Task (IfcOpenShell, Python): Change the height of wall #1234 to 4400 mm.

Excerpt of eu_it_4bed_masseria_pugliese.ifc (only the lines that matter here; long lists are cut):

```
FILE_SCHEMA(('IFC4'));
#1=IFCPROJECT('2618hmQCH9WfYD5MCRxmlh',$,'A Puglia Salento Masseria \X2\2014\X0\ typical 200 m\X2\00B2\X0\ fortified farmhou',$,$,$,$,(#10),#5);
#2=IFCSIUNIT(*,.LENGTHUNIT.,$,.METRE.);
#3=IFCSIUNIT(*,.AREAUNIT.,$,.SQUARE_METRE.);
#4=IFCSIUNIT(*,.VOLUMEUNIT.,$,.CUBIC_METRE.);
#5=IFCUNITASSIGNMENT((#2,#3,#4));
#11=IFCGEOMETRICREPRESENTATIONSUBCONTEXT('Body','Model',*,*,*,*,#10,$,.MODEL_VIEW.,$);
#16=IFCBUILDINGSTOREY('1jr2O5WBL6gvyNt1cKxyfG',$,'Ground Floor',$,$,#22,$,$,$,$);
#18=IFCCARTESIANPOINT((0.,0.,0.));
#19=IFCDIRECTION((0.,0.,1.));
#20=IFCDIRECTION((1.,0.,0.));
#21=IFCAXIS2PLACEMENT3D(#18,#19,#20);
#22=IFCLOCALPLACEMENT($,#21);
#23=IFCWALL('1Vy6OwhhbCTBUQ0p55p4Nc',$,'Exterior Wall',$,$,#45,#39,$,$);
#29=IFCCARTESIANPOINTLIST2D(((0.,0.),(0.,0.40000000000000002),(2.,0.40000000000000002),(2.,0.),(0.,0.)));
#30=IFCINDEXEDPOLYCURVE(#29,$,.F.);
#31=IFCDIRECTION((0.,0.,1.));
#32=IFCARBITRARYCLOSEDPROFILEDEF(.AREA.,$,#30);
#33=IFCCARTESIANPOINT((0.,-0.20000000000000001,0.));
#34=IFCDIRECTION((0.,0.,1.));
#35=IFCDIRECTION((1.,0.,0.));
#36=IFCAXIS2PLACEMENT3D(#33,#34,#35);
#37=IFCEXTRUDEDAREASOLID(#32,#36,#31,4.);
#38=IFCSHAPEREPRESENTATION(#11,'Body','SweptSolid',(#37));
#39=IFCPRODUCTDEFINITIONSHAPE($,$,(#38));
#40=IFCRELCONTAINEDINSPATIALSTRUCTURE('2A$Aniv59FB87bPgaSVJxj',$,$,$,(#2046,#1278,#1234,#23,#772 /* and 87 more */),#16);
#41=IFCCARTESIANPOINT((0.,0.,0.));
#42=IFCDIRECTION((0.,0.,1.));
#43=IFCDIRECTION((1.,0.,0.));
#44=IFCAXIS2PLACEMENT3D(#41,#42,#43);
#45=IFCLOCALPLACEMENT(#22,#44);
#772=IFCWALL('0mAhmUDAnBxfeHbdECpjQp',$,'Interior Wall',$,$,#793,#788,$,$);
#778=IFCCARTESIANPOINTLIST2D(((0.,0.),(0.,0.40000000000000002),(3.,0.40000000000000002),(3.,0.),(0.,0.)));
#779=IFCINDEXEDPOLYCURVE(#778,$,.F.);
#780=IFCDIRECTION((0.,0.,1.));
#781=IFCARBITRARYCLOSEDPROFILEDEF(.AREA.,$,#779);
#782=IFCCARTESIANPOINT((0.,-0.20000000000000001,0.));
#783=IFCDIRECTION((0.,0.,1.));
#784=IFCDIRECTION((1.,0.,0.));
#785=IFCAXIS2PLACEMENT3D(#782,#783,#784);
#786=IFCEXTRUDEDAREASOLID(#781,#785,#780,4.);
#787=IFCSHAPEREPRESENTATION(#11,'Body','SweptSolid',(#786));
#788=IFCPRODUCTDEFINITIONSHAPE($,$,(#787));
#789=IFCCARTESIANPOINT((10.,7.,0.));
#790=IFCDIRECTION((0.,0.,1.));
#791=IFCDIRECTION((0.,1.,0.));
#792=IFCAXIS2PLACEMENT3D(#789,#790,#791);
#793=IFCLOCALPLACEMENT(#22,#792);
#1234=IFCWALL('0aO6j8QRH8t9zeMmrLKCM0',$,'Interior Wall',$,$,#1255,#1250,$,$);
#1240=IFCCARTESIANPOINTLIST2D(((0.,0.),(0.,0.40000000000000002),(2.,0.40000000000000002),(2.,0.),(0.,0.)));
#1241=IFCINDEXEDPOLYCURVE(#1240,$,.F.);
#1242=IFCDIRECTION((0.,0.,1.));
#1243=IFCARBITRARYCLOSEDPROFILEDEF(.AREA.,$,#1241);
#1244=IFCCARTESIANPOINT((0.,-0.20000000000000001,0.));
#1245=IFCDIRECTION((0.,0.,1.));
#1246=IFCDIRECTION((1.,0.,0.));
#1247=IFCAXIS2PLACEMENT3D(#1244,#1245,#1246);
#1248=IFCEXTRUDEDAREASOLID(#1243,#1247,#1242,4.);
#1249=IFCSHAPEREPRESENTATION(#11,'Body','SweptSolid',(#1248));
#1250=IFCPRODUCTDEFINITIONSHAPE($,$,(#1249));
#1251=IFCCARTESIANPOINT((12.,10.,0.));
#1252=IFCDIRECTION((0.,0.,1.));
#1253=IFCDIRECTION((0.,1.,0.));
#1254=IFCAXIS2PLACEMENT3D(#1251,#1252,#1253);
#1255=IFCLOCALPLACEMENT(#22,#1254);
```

```python
import ifcopenshell
import ifcopenshell.geom
import ifcopenshell.util.representation
import ifcopenshell.util.shape
import ifcopenshell.util.unit

model = ifcopenshell.open("eu_it_4bed_masseria_pugliese.ifc")
unit_scale = ifcopenshell.util.unit.calculate_unit_scale(model)
settings = ifcopenshell.geom.settings()


def volume(element):
    """Net volume in cubic metres, openings subtracted."""
    shape = ifcopenshell.geom.create_shape(settings, element)
    return ifcopenshell.util.shape.get_volume(shape.geometry)


wall = model.by_guid("0aO6j8QRH8t9zeMmrLKCM0")
before = volume(wall)

body = ifcopenshell.util.representation.get_representation(wall, "Model", "Body")
solid = body.Items[0]
old_height = solid.Depth
solid.Depth = 4.4 / unit_scale
after = volume(wall)

print(f"height {old_height:g} -> {solid.Depth:g}, volume {before:.3f} -> {after:.3f} m3")

model.write("eu_it_4bed_masseria_pugliese_v2.ifc")
```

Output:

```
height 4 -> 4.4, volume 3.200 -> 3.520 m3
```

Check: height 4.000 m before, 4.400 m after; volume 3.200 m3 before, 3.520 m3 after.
